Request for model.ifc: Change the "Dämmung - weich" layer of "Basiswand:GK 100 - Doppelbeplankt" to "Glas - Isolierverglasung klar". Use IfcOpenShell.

First a look at what the model holds.

```python
import ifcopenshell
import ifcopenshell.util.element

model = ifcopenshell.open("model.ifc")
print(model.schema)
for layer_set in model.by_type("IfcMaterialLayerSet"):
    if layer_set.LayerSetName == "Basiswand:GK 100 - Doppelbeplankt":
        for layer in layer_set.MaterialLayers:
            print(layer.id(), layer.Material and layer.Material.Name, layer.LayerThickness, sep=" | ")
        print(len(ifcopenshell.util.element.get_elements_by_material(model, layer_set)), "elements and types use it")
print(sorted(m.Name for m in model.by_type("IfcMaterial") if m.Name)[:60])
```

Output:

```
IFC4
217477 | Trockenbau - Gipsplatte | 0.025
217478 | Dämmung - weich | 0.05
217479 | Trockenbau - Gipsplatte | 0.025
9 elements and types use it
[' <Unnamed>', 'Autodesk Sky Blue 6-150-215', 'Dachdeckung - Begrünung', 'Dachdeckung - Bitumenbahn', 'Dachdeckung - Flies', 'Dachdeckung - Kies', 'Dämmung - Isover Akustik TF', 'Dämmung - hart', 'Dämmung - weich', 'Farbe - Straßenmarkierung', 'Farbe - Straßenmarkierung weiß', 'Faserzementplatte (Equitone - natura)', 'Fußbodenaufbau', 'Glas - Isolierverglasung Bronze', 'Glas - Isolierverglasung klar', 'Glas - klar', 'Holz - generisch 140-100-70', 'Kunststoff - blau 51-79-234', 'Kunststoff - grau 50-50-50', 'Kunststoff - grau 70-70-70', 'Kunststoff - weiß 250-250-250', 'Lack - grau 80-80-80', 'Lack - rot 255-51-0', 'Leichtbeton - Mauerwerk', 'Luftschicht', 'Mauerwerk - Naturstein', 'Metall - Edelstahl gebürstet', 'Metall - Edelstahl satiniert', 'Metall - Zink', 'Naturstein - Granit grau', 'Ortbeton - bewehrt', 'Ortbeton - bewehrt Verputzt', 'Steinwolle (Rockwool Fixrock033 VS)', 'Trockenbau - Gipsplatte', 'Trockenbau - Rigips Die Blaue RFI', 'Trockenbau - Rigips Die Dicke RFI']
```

```python
import ifcopenshell
import ifcopenshell.api.material

model = ifcopenshell.open("model.ifc")

layer_set = next(s for s in model.by_type("IfcMaterialLayerSet") if s.LayerSetName == "Basiswand:GK 100 - Doppelbeplankt")
layer = next(l for l in layer_set.MaterialLayers if l.Material and l.Material.Name == "Dämmung - weich")
material = next(m for m in model.by_type("IfcMaterial") if m.Name == "Glas - Isolierverglasung klar")

# Point this one layer at the other material; renaming the old one would change it everywhere.
ifcopenshell.api.material.edit_layer(model, layer=layer, attributes={"Name": material.Name}, material=material)

print([l.Material.Name if l.Material else None for l in layer_set.MaterialLayers])

model.write("model_edited.ifc")
```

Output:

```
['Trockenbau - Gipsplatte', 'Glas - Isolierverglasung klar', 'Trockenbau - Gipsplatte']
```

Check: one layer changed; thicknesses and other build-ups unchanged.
